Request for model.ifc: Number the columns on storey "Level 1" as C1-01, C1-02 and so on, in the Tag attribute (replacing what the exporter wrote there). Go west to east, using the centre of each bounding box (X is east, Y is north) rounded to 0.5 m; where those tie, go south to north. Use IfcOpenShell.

First a look at what the model holds.

```python
import ifcopenshell
import ifcopenshell.util.element
import ifcopenshell.util.placement

model = ifcopenshell.open("model.ifc")
print(model.schema)
storey = next(s for s in model.by_type("IfcBuildingStorey") if s.Name == "Level 1")
columns = [e for e in ifcopenshell.util.element.get_decomposition(storey) if e.is_a("IfcColumn")]
for e in sorted(columns, key=lambda e: e.id()):
    origin = ifcopenshell.util.placement.get_local_placement(e.ObjectPlacement)[:3, 3]
    print(e.id(), e.Tag, e.Name, origin.round(2) + 0.0, sep=" | ")
```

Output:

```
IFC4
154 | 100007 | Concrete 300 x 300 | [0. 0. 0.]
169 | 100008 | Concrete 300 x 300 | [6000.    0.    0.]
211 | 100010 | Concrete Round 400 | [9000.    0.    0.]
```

```python
import ifcopenshell
import ifcopenshell.geom
import ifcopenshell.util.element
import ifcopenshell.util.shape

model = ifcopenshell.open("model.ifc")
settings = ifcopenshell.geom.settings()
settings.set("use-world-coords", True)


def centre(element):
    shape = ifcopenshell.geom.create_shape(settings, element)
    return ifcopenshell.util.shape.get_bbox_centroid(shape.geometry)


storey = next(s for s in model.by_type("IfcBuildingStorey") if s.Name == "Level 1")
columns = [e for e in ifcopenshell.util.element.get_decomposition(storey) if e.is_a("IfcColumn")]

# Insertion points can sit at a corner or the storey origin, so sort by the geometry (in metres).
centres = {e: centre(e) for e in columns}
columns.sort(key=lambda e: (round(centres[e][0] / 0.5), centres[e][1]))

for i, e in enumerate(columns, start=1):
    number = f"C1-{i:02d}"
    e.Tag = number
    print(e.id(), number)

model.write("model_rev.ifc")
```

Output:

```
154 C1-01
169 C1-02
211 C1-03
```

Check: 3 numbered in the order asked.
